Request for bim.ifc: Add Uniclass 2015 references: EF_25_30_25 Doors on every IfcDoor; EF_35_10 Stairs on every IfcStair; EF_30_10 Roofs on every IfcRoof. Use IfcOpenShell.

First a look at what the model holds.

```python
import ifcopenshell

model = ifcopenshell.open("bim.ifc")
print(model.schema)
print("classifications:", [c.Name for c in model.by_type("IfcClassification")])
for ifc_class in ("IfcDoor", "IfcRoof", "IfcStair", "IfcWall", "IfcWindow"):
    print(ifc_class, len(model.by_type(ifc_class)))
```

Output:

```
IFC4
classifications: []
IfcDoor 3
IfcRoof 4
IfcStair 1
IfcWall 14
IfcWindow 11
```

```python
import ifcopenshell
import ifcopenshell.api.classification

model = ifcopenshell.open("bim.ifc")

system = ifcopenshell.api.classification.add_classification(model, classification="Uniclass 2015")

codes = {
    "IfcDoor": ("EF_25_30_25", "Doors"),
    "IfcStair": ("EF_35_10", "Stairs"),
    "IfcRoof": ("EF_30_10", "Roofs"),
}
for ifc_class, (code, name) in codes.items():
    products = model.by_type(ifc_class)
    ifcopenshell.api.classification.add_reference(
        model, products=products, classification=system, identification=code, name=name
    )
    print(code, len(products))

model.write("bim_updated.ifc")
```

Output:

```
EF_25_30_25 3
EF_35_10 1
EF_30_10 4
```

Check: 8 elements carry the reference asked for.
